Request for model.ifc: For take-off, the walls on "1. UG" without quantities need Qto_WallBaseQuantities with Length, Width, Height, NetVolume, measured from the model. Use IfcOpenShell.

First a look at what the model holds.

```python
import ifcopenshell
import ifcopenshell.util.element
import ifcopenshell.util.unit

model = ifcopenshell.open("model.ifc")
print(model.schema)
for unit_type in ("LENGTHUNIT", "AREAUNIT", "VOLUMEUNIT"):
    print(unit_type, ifcopenshell.util.unit.calculate_unit_scale(model, unit_type))
storey = next(s for s in model.by_type("IfcBuildingStorey") if s.Name == "1. UG")
walls = [e for e in ifcopenshell.util.element.get_decomposition(storey) if e.is_a("IfcWall")]
for e in sorted(walls, key=lambda e: e.id()):
    print(e.id(), e.is_a(), e.Name, list(ifcopenshell.util.element.get_psets(e, qtos_only=True)), sep=" | ")
```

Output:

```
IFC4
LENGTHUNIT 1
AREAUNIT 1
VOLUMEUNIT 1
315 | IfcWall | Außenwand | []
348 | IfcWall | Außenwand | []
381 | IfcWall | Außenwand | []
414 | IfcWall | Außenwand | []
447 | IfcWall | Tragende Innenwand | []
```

```python
import ifcopenshell
import ifcopenshell.api.pset
import ifcopenshell.geom
import ifcopenshell.util.element
import ifcopenshell.util.shape
import ifcopenshell.util.unit

model = ifcopenshell.open("model.ifc")
unit_scale = ifcopenshell.util.unit.calculate_unit_scale(model)
volume_scale = ifcopenshell.util.unit.calculate_unit_scale(model, "VOLUMEUNIT")
settings = ifcopenshell.geom.settings()

storey = next(s for s in model.by_type("IfcBuildingStorey") if s.Name == "1. UG")
walls = [e for e in ifcopenshell.util.element.get_decomposition(storey) if e.is_a("IfcWall")]

for e in sorted(walls, key=lambda e: e.id()):
    if ifcopenshell.util.element.get_psets(e, qtos_only=True, should_inherit=False):
        continue
    # Geometry comes back in metres, in the element's own axes.
    shape = ifcopenshell.geom.create_shape(settings, e)
    values = {
        "Length": ifcopenshell.util.shape.get_x(shape.geometry) / unit_scale,
        "Width": ifcopenshell.util.shape.get_y(shape.geometry) / unit_scale,
        "Height": ifcopenshell.util.shape.get_z(shape.geometry) / unit_scale,
        "NetVolume": ifcopenshell.util.shape.get_volume(shape.geometry) / volume_scale,
    }
    qto = ifcopenshell.api.pset.add_qto(model, product=e, name="Qto_WallBaseQuantities")
    ifcopenshell.api.pset.edit_qto(model, qto=qto, properties=values)
    print(e.id(), {k: round(v, 3) for k, v in values.items()})

model.write("model_v2.ifc")
```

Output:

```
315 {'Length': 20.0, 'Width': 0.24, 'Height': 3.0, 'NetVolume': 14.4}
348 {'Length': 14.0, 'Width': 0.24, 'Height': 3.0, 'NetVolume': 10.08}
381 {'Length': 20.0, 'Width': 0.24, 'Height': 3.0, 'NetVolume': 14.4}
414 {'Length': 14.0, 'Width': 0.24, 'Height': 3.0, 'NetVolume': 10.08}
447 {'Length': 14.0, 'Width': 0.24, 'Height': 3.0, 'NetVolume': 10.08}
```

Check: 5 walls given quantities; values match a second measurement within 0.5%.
